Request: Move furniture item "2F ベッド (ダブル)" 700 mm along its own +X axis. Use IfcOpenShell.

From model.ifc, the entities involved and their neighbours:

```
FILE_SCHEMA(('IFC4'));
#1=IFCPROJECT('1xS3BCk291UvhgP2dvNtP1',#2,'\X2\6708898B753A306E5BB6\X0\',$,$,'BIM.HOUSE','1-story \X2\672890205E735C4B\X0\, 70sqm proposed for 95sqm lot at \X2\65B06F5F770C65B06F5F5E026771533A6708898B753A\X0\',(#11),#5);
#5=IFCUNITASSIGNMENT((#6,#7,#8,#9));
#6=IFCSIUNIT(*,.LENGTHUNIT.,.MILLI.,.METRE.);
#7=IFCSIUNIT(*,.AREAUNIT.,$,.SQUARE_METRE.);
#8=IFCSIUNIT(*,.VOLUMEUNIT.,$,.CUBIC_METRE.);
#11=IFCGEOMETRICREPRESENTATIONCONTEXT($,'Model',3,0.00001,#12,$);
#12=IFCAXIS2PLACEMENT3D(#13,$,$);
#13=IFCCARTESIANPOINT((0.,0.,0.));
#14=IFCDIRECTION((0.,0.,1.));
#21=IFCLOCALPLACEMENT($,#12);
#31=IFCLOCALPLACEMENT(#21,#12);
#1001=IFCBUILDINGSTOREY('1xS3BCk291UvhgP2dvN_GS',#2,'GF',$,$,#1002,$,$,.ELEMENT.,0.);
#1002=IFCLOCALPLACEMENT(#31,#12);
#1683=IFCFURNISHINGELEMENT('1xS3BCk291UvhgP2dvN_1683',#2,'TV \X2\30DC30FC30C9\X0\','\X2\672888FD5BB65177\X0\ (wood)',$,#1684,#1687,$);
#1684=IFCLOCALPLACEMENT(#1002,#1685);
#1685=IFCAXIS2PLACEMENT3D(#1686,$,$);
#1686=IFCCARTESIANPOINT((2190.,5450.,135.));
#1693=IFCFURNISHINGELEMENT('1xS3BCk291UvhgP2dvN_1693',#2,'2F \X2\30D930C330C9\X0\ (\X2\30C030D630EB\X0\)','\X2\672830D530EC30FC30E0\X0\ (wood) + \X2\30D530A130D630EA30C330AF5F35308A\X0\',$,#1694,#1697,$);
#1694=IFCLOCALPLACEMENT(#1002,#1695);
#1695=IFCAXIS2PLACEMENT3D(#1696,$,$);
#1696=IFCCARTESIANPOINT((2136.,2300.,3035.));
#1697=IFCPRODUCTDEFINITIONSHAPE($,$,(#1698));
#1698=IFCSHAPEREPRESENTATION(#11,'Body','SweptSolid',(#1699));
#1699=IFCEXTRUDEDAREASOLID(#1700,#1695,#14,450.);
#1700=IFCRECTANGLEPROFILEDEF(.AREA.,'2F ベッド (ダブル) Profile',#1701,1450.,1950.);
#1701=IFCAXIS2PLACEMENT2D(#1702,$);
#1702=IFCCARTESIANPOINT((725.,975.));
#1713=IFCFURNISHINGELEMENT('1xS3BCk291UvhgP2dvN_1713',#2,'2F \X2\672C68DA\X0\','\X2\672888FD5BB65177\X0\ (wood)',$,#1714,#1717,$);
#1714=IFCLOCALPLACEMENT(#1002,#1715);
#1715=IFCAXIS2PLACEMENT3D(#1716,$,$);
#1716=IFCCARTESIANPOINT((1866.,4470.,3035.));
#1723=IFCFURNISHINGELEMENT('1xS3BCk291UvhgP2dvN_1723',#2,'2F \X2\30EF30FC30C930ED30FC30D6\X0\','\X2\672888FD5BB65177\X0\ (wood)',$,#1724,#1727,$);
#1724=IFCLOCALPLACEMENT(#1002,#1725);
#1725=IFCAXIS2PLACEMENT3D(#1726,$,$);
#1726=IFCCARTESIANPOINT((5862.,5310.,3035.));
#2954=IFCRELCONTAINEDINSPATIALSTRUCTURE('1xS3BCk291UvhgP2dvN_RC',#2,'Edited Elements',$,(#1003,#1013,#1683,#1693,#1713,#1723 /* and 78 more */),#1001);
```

```python
import ifcopenshell
import ifcopenshell.api.geometry
import ifcopenshell.util.placement

model = ifcopenshell.open("model.ifc")

item = model.by_guid("1xS3BCk291UvhgP2dvN_1693")
matrix = ifcopenshell.util.placement.get_local_placement(item.ObjectPlacement)
matrix[:3, 3] += matrix[:3, 0] * 700.0
ifcopenshell.api.geometry.edit_object_placement(model, product=item, matrix=matrix, is_si=False)

print(ifcopenshell.util.placement.get_local_placement(item.ObjectPlacement).round(3) + 0.0)

model.write("model_updated.ifc")
```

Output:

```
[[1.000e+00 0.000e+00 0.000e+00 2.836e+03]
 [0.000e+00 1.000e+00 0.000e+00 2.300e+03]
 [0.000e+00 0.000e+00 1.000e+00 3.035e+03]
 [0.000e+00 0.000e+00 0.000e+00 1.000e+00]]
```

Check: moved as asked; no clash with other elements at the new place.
